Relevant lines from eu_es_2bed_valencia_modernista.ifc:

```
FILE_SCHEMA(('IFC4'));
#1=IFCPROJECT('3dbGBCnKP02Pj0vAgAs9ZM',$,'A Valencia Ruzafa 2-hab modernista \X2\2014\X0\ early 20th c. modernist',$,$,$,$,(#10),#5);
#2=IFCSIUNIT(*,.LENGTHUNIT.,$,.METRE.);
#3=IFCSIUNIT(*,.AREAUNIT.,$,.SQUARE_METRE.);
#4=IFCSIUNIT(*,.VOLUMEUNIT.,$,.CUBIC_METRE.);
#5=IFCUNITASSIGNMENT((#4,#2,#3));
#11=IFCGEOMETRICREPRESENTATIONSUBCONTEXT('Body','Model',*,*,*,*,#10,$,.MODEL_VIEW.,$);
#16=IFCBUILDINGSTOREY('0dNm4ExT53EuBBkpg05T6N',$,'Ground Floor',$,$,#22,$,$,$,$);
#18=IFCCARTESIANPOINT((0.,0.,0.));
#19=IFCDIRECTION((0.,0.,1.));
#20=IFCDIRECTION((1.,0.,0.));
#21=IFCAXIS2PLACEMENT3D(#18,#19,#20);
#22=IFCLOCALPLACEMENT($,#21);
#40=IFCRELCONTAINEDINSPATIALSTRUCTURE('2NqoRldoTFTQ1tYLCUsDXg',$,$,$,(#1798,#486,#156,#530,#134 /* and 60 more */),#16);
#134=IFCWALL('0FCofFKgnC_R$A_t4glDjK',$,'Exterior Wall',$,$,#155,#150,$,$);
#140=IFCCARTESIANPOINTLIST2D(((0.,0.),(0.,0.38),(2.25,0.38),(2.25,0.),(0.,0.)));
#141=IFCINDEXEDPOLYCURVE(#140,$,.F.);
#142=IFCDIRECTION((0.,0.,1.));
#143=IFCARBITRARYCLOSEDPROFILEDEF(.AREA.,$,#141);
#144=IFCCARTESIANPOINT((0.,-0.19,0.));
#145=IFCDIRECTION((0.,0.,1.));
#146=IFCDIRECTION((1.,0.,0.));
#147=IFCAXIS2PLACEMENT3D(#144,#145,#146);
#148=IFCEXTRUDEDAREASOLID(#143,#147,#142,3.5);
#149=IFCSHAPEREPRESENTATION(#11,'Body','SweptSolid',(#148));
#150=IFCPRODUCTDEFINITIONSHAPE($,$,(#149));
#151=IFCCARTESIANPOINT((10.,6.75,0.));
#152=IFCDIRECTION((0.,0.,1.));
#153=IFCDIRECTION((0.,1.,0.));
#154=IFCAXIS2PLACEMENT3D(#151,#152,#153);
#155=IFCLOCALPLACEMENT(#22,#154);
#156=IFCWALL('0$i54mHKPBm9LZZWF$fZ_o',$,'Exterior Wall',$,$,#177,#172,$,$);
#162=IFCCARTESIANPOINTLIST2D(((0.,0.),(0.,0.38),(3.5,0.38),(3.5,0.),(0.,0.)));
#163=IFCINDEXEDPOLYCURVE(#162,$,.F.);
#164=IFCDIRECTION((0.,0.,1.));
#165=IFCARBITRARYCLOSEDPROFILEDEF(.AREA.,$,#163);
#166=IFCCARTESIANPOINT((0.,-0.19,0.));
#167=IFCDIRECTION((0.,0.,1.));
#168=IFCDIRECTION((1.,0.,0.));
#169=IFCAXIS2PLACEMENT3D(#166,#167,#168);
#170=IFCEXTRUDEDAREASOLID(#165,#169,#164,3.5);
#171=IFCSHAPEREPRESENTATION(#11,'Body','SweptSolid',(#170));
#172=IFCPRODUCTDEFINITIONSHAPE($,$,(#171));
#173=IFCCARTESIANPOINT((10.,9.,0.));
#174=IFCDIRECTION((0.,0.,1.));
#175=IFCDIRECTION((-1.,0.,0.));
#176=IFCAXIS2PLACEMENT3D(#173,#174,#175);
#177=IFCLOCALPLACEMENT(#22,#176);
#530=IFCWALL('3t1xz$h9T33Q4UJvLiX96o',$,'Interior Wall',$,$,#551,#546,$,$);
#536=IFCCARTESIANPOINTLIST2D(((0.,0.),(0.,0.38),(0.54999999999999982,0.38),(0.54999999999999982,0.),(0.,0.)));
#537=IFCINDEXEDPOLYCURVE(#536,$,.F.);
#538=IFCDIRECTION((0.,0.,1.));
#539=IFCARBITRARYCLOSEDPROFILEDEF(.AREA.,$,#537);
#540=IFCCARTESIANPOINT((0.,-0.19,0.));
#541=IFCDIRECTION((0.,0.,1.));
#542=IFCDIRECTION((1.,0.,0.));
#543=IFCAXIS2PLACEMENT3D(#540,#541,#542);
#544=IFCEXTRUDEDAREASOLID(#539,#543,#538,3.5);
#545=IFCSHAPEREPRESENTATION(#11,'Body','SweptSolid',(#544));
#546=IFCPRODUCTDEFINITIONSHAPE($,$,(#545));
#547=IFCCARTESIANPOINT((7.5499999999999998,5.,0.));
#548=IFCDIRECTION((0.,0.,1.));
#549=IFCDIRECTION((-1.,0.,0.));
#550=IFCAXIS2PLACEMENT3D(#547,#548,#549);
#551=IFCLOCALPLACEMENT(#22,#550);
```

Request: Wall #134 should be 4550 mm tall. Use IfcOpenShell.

```python
import ifcopenshell
import ifcopenshell.geom
import ifcopenshell.util.representation
import ifcopenshell.util.shape
import ifcopenshell.util.unit

model = ifcopenshell.open("eu_es_2bed_valencia_modernista.ifc")
unit_scale = ifcopenshell.util.unit.calculate_unit_scale(model)
settings = ifcopenshell.geom.settings()


def volume(element):
    """Net volume in cubic metres, openings subtracted."""
    shape = ifcopenshell.geom.create_shape(settings, element)
    return ifcopenshell.util.shape.get_volume(shape.geometry)


wall = model.by_id(134)
before = volume(wall)

body = ifcopenshell.util.representation.get_representation(wall, "Model", "Body")
solid = body.Items[0]
old_height = solid.Depth
solid.Depth = 4.55 / unit_scale
after = volume(wall)

print(f"height {old_height:g} -> {solid.Depth:g}, volume {before:.3f} -> {after:.3f} m3")

model.write("eu_es_2bed_valencia_modernista_rev.ifc")
```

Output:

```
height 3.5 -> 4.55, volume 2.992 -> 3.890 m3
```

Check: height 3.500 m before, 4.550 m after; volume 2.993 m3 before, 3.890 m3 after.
